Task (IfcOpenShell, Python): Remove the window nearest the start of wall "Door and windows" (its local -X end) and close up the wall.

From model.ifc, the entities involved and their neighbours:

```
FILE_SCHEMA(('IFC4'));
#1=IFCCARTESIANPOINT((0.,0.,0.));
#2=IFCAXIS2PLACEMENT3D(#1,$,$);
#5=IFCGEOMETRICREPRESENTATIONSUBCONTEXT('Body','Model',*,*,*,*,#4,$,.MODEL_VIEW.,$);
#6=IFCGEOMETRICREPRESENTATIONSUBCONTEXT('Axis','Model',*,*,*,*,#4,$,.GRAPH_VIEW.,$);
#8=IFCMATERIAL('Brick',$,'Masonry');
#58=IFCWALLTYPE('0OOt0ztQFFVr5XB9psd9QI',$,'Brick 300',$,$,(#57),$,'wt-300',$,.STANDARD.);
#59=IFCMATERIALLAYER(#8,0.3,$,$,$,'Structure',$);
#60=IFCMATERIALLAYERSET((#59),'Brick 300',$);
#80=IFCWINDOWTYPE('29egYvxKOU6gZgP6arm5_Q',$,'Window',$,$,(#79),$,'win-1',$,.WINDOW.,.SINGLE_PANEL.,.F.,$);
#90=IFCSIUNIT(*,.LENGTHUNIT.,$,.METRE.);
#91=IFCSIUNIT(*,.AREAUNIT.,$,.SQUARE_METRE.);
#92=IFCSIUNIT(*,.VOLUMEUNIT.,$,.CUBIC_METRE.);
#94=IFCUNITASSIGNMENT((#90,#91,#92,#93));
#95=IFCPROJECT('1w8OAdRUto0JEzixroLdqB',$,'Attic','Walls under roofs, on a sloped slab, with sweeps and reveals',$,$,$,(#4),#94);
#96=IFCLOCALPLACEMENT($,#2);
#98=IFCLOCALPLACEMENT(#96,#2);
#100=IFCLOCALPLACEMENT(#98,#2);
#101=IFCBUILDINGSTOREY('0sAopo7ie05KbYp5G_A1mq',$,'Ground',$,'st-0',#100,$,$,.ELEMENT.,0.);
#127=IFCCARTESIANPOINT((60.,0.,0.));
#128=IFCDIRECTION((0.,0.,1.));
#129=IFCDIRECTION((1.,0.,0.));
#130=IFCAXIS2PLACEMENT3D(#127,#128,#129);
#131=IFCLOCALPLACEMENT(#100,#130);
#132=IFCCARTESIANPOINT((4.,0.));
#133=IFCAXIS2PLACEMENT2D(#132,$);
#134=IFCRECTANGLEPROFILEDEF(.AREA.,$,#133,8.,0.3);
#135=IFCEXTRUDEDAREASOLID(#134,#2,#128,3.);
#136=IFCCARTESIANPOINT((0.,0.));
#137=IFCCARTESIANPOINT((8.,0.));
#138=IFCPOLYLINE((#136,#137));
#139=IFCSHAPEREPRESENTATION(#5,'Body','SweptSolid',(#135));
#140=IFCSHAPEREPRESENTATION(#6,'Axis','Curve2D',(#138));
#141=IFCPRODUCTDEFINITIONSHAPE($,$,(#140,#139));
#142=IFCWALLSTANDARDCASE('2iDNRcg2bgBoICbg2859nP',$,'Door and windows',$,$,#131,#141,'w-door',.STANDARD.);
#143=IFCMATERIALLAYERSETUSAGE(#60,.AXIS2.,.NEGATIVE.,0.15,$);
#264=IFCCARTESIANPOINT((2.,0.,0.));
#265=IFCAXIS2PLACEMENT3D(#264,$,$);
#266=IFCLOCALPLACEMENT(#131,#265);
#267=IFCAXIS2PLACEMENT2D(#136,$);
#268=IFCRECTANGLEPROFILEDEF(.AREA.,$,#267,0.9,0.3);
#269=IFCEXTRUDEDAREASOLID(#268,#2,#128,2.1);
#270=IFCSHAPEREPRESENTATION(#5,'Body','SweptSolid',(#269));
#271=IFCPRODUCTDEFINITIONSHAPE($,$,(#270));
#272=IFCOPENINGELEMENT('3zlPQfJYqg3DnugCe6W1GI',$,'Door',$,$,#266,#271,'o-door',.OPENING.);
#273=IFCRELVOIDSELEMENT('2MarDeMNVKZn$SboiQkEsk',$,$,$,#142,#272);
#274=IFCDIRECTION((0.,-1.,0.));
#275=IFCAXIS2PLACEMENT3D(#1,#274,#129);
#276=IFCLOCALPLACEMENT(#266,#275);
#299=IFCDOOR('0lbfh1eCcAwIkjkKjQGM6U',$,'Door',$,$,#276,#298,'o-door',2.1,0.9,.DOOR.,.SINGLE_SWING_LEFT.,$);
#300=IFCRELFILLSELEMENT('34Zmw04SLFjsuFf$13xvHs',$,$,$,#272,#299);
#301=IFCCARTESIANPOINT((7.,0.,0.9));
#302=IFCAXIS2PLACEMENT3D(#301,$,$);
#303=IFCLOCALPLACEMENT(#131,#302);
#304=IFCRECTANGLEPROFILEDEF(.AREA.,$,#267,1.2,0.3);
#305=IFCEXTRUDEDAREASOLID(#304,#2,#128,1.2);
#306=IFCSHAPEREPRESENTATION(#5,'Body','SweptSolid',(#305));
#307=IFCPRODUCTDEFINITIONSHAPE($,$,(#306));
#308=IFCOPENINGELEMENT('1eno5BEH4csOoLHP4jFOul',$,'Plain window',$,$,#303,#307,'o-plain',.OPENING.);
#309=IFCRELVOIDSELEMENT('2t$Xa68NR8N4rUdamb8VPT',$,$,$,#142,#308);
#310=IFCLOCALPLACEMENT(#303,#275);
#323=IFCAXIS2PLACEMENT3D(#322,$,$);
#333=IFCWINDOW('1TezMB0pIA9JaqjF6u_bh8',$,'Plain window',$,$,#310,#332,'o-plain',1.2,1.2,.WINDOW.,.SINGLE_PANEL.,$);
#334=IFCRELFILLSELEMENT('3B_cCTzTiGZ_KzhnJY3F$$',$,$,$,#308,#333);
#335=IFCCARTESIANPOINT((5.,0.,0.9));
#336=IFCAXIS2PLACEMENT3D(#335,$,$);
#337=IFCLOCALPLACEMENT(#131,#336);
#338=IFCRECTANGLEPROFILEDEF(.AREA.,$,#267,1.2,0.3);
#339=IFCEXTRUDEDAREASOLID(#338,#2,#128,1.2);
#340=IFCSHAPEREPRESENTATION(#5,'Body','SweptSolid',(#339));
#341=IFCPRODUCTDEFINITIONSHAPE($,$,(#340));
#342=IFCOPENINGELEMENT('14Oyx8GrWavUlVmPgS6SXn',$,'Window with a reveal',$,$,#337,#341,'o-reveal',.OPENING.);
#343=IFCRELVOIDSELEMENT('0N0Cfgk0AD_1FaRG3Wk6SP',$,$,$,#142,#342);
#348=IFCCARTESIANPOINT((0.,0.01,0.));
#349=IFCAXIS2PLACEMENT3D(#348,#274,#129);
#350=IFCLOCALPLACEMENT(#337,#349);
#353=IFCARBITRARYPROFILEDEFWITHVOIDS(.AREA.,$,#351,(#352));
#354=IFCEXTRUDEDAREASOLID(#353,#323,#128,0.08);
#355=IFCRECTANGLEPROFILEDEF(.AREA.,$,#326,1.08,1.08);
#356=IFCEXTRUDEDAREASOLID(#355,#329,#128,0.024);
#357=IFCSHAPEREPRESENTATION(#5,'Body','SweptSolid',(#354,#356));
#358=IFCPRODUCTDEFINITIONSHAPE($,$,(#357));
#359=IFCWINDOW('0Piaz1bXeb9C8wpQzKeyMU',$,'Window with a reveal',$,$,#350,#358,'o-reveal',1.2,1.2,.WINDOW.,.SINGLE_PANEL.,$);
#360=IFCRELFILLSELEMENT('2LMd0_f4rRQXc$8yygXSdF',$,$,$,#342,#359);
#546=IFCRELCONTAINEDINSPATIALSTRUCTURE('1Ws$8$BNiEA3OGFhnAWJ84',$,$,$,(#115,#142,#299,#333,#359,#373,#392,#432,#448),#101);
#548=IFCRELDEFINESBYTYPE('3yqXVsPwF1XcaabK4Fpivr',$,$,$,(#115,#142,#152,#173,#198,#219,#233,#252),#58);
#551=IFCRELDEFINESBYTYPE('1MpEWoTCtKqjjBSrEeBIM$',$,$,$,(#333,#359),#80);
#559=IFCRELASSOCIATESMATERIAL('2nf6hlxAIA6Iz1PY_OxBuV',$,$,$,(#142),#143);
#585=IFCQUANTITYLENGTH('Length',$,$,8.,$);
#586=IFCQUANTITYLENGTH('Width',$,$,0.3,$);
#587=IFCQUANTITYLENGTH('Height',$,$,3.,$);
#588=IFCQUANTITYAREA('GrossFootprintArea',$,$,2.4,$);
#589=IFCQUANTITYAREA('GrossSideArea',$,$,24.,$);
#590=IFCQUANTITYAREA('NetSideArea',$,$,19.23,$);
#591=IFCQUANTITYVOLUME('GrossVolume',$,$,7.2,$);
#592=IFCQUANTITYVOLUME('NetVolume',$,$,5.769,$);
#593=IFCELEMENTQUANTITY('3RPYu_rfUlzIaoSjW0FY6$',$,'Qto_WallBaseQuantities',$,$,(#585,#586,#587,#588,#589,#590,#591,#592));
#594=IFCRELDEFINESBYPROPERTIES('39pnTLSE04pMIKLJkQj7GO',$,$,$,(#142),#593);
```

```python
import ifcopenshell
import ifcopenshell.api.feature
import ifcopenshell.api.pset
import ifcopenshell.api.root
import ifcopenshell.geom
import ifcopenshell.util.element
import ifcopenshell.util.shape
import ifcopenshell.util.unit

model = ifcopenshell.open("model.ifc")
area_scale = ifcopenshell.util.unit.calculate_unit_scale(model, "AREAUNIT")
volume_scale = ifcopenshell.util.unit.calculate_unit_scale(model, "VOLUMEUNIT")
settings = ifcopenshell.geom.settings()


def volume(element):
    """Net volume in cubic metres, openings subtracted."""
    shape = ifcopenshell.geom.create_shape(settings, element)
    return ifcopenshell.util.shape.get_volume(shape.geometry)


window = model.by_guid("0Piaz1bXeb9C8wpQzKeyMU")
opening = window.FillsVoids[0].RelatingOpeningElement
wall = opening.VoidsElements[0].RelatingBuildingElement
before = volume(wall)

ifcopenshell.api.root.remove_product(model, product=window)
ifcopenshell.api.feature.remove_feature(model, feature=opening)

after = volume(wall)
thickness = 0.3  # wall thickness in metres

# Update the wall's stored quantities.
qto = model.by_id(ifcopenshell.util.element.get_pset(wall, "Qto_WallBaseQuantities", should_inherit=False)["id"])
ifcopenshell.api.pset.edit_qto(model, qto=qto, properties={
    "NetSideArea": after / thickness / area_scale,
    "NetVolume": after / volume_scale,
})

print(f"wall volume {before:.3f} -> {after:.3f} m3")

model.write("model-out.ifc")
```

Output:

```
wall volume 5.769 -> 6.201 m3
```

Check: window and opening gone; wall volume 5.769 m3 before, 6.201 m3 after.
